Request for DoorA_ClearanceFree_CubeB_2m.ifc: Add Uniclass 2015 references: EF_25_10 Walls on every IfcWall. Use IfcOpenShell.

First a look at what the model holds.

```python
import ifcopenshell

model = ifcopenshell.open("DoorA_ClearanceFree_CubeB_2m.ifc")
print(model.schema)
print("classifications:", [c.Name for c in model.by_type("IfcClassification")])
for ifc_class in ("IfcDoor", "IfcRoof", "IfcStair", "IfcWall", "IfcWindow"):
    print(ifc_class, len(model.by_type(ifc_class)))
```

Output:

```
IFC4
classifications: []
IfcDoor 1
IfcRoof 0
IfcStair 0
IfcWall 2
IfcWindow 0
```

```python
import ifcopenshell
import ifcopenshell.api.classification

model = ifcopenshell.open("DoorA_ClearanceFree_CubeB_2m.ifc")

system = ifcopenshell.api.classification.add_classification(model, classification="Uniclass 2015")

codes = {
    "IfcWall": ("EF_25_10", "Walls"),
}
for ifc_class, (code, name) in codes.items():
    products = model.by_type(ifc_class)
    ifcopenshell.api.classification.add_reference(
        model, products=products, classification=system, identification=code, name=name
    )
    print(code, len(products))

model.write("DoorA_ClearanceFree_CubeB_2m_updated.ifc")
```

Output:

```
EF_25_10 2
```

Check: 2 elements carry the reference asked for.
